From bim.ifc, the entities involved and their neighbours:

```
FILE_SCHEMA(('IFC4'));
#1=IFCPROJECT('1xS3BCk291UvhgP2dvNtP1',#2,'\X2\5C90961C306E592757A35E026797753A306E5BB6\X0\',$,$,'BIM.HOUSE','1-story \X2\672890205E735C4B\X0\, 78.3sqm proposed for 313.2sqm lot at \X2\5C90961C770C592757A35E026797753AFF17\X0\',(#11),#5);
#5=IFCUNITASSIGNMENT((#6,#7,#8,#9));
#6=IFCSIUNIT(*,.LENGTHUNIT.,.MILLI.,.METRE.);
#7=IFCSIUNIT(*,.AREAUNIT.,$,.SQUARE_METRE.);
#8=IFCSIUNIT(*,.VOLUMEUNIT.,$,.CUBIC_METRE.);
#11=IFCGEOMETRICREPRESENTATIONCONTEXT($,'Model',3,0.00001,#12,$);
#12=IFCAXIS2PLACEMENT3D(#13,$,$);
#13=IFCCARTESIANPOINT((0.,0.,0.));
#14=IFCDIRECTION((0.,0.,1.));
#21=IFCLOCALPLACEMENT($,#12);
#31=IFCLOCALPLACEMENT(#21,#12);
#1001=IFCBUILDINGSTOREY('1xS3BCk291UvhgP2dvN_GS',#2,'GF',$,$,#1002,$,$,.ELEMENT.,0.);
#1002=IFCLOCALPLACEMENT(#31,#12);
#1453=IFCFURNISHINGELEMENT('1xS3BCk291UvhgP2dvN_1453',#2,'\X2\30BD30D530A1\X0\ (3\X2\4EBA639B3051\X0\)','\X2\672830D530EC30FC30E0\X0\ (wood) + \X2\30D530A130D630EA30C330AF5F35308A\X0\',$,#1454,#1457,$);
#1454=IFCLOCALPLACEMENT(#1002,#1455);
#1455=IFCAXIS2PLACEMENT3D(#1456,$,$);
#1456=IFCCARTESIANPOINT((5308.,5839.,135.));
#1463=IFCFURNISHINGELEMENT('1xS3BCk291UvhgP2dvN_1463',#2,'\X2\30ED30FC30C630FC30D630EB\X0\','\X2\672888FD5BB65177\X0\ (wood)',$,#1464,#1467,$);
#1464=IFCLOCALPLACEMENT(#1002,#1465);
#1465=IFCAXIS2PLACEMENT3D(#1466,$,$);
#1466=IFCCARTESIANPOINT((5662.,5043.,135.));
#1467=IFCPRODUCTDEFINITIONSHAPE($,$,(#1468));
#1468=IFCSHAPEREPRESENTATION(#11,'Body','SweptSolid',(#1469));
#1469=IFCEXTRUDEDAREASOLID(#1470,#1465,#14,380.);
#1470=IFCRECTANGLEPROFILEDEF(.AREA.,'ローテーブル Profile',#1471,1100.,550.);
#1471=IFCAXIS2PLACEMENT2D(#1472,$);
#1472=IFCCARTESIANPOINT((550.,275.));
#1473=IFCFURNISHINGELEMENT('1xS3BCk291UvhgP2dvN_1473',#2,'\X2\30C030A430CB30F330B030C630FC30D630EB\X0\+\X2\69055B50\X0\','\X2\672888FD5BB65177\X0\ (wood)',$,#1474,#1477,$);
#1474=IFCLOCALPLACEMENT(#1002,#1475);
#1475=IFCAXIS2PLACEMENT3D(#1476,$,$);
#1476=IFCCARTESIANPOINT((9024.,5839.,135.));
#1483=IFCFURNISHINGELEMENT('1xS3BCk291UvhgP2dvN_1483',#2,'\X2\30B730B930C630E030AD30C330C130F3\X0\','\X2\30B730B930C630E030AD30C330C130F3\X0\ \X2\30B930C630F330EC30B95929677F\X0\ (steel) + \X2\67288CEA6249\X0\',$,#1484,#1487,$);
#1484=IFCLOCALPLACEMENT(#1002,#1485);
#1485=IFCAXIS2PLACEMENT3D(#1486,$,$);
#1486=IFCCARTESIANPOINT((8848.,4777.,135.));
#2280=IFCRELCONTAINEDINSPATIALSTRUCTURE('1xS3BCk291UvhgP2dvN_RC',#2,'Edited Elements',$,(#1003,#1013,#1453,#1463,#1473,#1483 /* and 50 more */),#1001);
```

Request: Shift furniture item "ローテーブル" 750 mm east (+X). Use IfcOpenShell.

```python
import ifcopenshell
import ifcopenshell.api.geometry
import ifcopenshell.util.placement
import ifcopenshell.util.unit

model = ifcopenshell.open("bim.ifc")
unit_scale = ifcopenshell.util.unit.calculate_unit_scale(model)

item = model.by_guid("1xS3BCk291UvhgP2dvN_1463")
matrix = ifcopenshell.util.placement.get_local_placement(item.ObjectPlacement)
matrix[0, 3] += 0.75 / unit_scale
ifcopenshell.api.geometry.edit_object_placement(model, product=item, matrix=matrix, is_si=False)

print(ifcopenshell.util.placement.get_local_placement(item.ObjectPlacement).round(3) + 0.0)

model.write("bim-out.ifc")
```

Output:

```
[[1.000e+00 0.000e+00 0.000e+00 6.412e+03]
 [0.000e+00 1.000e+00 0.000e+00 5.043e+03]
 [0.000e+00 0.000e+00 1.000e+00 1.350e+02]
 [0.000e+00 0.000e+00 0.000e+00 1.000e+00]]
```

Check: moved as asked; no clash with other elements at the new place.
